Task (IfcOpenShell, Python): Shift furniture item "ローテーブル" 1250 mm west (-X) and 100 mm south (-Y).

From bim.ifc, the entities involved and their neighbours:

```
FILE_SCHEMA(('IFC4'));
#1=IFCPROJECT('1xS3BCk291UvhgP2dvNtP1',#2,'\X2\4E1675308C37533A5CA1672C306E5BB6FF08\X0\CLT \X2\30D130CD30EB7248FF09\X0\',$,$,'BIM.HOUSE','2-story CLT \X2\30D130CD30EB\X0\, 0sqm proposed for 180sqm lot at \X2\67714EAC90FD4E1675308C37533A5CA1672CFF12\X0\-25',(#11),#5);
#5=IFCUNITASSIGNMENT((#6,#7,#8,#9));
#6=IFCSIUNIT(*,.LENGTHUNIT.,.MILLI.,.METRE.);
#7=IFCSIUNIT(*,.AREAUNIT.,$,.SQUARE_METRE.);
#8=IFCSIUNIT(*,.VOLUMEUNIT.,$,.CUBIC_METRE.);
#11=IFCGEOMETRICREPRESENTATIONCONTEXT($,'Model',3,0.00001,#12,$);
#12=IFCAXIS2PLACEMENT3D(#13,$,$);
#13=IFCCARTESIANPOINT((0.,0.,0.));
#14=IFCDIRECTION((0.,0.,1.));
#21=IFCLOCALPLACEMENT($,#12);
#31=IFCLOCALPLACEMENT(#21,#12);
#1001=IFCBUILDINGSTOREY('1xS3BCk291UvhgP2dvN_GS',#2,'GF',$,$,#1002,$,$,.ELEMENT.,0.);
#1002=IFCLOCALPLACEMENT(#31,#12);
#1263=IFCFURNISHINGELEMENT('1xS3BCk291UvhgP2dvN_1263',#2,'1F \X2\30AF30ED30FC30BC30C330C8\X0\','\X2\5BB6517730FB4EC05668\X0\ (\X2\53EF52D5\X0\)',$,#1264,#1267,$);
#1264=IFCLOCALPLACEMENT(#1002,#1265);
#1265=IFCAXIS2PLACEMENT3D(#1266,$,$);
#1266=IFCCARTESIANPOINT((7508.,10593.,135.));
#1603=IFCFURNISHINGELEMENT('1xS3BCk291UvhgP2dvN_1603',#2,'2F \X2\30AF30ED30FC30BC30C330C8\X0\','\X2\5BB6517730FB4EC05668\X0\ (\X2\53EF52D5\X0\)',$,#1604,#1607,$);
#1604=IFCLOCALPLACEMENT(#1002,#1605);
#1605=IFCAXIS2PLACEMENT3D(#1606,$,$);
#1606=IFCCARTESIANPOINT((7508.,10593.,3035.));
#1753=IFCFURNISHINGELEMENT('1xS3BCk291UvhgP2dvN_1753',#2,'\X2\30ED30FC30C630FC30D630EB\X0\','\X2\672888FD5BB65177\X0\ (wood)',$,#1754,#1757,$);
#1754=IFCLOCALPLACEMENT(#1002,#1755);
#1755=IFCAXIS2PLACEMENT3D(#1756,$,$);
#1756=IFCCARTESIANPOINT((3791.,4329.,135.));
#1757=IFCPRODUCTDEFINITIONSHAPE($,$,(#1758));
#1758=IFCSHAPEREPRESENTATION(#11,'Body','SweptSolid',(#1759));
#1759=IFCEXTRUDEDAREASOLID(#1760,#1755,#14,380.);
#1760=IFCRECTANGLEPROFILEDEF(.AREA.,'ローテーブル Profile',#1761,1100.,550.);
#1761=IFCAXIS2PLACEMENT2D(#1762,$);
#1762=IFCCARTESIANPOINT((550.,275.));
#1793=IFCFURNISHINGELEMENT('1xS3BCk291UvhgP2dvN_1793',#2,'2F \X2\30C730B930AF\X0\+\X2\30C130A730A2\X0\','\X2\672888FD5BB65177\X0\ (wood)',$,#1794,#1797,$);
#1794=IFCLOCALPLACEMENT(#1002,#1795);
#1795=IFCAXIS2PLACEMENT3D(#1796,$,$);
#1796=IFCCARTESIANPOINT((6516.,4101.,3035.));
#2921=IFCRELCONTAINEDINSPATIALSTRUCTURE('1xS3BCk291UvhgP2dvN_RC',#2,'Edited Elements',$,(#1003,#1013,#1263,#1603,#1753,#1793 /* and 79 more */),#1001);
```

```python
import ifcopenshell
import ifcopenshell.api.geometry
import ifcopenshell.util.placement
import ifcopenshell.util.unit

model = ifcopenshell.open("bim.ifc")
unit_scale = ifcopenshell.util.unit.calculate_unit_scale(model)

item = model.by_guid("1xS3BCk291UvhgP2dvN_1753")
matrix = ifcopenshell.util.placement.get_local_placement(item.ObjectPlacement)
matrix[0, 3] -= 1.25 / unit_scale
matrix[1, 3] -= 0.1 / unit_scale
ifcopenshell.api.geometry.edit_object_placement(model, product=item, matrix=matrix, is_si=False)

print(ifcopenshell.util.placement.get_local_placement(item.ObjectPlacement).round(3) + 0.0)

model.write("bim_edited.ifc")
```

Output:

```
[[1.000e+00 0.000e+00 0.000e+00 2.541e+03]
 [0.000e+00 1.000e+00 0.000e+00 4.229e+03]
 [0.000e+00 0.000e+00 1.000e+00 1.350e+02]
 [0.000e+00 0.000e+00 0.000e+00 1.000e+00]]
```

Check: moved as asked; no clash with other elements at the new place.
